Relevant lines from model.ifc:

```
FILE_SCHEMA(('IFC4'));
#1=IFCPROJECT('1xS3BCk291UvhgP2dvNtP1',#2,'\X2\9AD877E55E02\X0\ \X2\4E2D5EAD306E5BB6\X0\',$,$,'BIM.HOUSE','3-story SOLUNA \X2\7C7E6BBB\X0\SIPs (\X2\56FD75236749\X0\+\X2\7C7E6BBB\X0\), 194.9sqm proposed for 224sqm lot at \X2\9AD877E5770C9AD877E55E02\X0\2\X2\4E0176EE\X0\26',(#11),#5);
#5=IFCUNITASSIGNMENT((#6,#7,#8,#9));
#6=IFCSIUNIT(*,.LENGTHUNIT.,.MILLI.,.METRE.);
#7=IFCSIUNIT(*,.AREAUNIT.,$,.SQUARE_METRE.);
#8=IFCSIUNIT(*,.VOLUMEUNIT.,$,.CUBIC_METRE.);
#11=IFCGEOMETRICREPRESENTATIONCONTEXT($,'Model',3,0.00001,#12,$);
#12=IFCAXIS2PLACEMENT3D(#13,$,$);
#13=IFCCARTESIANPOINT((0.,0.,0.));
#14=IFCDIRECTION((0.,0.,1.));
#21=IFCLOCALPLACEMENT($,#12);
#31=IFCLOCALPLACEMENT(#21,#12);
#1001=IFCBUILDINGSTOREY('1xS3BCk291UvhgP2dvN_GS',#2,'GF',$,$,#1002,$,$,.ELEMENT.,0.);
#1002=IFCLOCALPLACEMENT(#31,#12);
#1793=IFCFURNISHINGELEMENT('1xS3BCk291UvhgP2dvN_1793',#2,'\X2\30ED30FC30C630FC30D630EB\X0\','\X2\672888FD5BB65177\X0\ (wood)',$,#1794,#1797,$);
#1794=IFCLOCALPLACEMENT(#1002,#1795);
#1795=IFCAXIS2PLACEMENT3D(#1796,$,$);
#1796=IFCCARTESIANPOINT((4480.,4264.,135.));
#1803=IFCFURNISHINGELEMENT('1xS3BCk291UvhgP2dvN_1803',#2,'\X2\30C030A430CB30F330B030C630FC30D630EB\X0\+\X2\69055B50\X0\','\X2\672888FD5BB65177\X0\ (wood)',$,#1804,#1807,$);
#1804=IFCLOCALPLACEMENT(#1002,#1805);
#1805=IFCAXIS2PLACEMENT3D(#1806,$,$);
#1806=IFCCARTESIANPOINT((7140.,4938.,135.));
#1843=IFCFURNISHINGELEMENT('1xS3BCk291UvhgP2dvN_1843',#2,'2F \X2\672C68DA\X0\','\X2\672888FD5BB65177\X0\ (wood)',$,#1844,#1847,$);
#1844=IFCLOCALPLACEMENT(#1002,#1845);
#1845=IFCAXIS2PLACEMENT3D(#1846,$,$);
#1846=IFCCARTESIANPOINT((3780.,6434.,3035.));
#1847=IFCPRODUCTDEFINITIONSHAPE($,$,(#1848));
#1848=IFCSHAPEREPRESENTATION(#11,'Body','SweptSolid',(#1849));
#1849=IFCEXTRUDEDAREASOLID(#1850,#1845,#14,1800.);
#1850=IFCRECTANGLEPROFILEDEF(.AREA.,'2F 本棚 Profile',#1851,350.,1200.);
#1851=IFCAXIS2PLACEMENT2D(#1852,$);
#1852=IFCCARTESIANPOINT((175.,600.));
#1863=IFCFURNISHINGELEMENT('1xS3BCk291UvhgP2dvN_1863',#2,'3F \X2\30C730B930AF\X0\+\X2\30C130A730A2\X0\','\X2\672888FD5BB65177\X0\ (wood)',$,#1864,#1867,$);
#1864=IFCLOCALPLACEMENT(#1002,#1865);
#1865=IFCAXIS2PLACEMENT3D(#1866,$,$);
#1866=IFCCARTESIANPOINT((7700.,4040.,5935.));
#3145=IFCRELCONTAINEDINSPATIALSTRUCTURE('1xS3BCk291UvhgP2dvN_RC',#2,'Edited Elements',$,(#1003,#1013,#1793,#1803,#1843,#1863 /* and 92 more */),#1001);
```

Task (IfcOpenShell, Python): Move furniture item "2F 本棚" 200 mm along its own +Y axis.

```python
import ifcopenshell
import ifcopenshell.api.geometry
import ifcopenshell.util.placement
import ifcopenshell.util.unit

model = ifcopenshell.open("model.ifc")
unit_scale = ifcopenshell.util.unit.calculate_unit_scale(model)

item = model.by_guid("1xS3BCk291UvhgP2dvN_1843")
matrix = ifcopenshell.util.placement.get_local_placement(item.ObjectPlacement)
matrix[:3, 3] += matrix[:3, 1] * 0.2 / unit_scale
ifcopenshell.api.geometry.edit_object_placement(model, product=item, matrix=matrix, is_si=False)

print(ifcopenshell.util.placement.get_local_placement(item.ObjectPlacement).round(3) + 0.0)

model.write("model_rev.ifc")
```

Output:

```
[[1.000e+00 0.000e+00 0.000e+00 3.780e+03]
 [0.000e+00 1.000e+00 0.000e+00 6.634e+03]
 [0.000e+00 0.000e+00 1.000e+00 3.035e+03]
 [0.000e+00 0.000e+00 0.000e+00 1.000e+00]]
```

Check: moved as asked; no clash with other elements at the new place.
